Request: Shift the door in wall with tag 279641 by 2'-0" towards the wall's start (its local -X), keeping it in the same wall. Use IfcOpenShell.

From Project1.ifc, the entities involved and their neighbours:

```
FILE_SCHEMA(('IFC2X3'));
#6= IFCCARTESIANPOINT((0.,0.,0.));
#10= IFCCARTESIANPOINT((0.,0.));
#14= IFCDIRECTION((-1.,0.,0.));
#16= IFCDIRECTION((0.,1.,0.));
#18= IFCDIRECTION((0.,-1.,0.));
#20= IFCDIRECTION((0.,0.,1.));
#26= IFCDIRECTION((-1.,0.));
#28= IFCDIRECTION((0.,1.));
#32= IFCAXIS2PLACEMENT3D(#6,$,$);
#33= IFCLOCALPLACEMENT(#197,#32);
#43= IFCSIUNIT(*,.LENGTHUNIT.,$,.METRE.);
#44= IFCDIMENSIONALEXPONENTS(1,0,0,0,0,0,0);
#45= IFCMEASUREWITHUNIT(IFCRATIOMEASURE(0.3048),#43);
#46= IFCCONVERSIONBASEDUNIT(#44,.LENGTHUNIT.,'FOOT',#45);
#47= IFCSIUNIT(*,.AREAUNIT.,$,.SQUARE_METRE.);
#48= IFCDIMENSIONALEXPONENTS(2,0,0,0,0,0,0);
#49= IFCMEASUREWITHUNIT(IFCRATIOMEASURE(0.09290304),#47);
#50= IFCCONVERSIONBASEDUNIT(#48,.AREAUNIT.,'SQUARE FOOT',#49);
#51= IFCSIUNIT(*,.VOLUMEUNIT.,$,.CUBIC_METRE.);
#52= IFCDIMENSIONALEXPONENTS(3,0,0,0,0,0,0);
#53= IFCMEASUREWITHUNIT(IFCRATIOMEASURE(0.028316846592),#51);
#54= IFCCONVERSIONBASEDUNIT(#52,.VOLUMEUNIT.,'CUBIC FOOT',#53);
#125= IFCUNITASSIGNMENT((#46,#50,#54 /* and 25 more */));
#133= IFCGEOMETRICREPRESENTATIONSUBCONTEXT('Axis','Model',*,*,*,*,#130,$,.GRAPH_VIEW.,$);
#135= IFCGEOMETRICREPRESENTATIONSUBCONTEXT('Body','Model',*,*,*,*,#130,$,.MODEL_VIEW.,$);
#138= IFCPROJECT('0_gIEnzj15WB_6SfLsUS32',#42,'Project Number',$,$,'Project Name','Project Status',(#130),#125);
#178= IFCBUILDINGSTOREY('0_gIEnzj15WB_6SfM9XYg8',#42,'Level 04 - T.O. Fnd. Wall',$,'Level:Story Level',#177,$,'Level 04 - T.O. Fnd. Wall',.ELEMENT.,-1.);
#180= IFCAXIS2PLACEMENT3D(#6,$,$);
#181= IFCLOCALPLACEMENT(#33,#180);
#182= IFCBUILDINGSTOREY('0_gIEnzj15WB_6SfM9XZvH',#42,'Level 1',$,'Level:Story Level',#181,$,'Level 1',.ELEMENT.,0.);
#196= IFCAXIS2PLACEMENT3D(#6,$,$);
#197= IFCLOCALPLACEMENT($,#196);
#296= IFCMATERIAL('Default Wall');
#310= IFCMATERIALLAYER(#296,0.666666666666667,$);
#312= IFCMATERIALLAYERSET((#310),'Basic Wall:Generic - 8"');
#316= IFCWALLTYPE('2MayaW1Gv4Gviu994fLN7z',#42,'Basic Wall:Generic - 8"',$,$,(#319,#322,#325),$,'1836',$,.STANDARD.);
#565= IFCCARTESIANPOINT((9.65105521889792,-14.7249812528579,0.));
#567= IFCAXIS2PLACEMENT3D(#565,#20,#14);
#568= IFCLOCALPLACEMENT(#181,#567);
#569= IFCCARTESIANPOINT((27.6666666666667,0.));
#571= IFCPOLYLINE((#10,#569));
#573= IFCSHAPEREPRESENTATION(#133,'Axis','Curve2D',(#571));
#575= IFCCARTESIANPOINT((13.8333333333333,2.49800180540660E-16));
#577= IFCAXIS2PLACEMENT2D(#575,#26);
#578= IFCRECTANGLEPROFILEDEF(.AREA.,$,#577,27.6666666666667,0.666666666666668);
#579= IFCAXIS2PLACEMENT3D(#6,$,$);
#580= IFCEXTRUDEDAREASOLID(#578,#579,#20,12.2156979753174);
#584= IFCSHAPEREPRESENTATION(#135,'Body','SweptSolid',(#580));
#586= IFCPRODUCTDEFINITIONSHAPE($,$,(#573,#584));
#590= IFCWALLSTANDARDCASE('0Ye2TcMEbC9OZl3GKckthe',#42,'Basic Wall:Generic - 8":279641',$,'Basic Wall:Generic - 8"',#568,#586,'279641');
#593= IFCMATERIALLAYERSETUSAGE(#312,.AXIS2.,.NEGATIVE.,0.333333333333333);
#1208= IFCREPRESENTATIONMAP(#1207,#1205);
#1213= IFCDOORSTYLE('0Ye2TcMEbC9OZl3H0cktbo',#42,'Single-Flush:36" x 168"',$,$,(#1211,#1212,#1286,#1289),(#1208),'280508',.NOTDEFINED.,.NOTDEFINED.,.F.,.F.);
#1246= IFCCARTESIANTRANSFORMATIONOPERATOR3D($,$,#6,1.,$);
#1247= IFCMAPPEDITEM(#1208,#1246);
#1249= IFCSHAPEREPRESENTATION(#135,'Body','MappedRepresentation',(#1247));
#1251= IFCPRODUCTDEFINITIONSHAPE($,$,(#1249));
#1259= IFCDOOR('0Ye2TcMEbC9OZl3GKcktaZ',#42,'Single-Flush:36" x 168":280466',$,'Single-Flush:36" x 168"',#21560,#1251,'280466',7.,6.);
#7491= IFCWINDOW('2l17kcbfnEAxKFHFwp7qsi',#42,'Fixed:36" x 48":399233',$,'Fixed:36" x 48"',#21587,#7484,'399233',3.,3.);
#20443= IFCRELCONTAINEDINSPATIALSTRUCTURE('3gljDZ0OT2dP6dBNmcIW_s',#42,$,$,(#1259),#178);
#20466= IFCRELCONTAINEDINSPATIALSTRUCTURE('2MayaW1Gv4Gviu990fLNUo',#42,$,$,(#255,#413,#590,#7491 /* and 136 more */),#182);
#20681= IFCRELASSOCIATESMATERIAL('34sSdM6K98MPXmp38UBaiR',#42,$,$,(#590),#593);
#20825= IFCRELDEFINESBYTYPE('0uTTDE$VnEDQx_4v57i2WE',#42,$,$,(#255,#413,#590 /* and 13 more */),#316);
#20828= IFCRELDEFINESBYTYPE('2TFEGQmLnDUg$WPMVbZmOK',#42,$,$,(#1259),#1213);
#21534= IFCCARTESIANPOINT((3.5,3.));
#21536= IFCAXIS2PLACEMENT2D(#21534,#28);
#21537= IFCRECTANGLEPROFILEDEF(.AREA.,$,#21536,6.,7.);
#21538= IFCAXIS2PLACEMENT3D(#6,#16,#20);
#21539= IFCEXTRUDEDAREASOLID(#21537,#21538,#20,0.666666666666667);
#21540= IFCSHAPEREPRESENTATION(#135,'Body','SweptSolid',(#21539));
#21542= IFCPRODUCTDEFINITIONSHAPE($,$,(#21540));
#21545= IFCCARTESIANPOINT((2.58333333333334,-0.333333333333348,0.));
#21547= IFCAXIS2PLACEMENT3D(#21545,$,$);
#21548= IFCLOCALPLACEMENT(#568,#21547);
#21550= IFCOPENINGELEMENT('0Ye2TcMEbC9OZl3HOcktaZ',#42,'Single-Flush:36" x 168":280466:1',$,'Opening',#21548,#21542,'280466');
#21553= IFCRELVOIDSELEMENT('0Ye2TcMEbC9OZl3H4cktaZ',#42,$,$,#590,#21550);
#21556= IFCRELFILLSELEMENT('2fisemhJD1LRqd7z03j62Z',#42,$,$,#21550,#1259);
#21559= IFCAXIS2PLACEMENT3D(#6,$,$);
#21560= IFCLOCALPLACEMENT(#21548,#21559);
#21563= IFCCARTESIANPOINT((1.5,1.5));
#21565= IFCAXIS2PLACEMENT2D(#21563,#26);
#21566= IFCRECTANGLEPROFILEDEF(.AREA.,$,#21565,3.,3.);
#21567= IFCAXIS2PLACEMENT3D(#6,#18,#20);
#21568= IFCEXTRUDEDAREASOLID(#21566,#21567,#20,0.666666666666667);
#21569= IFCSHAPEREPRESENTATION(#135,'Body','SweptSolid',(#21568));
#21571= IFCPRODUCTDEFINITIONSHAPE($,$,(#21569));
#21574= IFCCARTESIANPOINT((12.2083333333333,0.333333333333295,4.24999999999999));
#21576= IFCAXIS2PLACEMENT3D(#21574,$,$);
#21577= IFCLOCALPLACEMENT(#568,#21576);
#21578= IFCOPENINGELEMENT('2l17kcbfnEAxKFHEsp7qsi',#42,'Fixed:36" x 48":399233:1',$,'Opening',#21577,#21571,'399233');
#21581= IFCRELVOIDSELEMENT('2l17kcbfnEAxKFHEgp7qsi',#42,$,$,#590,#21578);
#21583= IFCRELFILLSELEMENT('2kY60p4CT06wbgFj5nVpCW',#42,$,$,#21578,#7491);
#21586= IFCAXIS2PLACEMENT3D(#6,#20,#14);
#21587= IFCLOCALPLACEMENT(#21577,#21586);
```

```python
import ifcopenshell
import ifcopenshell.api.geometry
import ifcopenshell.util.placement
import ifcopenshell.util.unit

model = ifcopenshell.open("Project1.ifc")
unit_scale = ifcopenshell.util.unit.calculate_unit_scale(model)

door = model.by_guid("0Ye2TcMEbC9OZl3GKcktaZ")
opening = door.FillsVoids[0].RelatingOpeningElement
wall = opening.VoidsElements[0].RelatingBuildingElement

wall_matrix = ifcopenshell.util.placement.get_local_placement(wall.ObjectPlacement)
shift = wall_matrix[:3, 0] * -24 * 0.0254 / unit_scale
before = ifcopenshell.util.placement.get_local_placement(door.ObjectPlacement)[:3, 3].copy()

# The door is placed relative to its opening, so it follows when the opening moves.
matrix = ifcopenshell.util.placement.get_local_placement(opening.ObjectPlacement)
matrix[:3, 3] += shift
ifcopenshell.api.geometry.edit_object_placement(
    model, product=opening, matrix=matrix, is_si=False, should_transform_children=True
)

after = ifcopenshell.util.placement.get_local_placement(door.ObjectPlacement)[:3, 3]
print("door moved by", (after - before).round(3) + 0.0)

model.write("Project1_edited.ifc")
```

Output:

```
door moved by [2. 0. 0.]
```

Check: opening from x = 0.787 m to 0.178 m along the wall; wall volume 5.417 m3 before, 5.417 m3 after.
